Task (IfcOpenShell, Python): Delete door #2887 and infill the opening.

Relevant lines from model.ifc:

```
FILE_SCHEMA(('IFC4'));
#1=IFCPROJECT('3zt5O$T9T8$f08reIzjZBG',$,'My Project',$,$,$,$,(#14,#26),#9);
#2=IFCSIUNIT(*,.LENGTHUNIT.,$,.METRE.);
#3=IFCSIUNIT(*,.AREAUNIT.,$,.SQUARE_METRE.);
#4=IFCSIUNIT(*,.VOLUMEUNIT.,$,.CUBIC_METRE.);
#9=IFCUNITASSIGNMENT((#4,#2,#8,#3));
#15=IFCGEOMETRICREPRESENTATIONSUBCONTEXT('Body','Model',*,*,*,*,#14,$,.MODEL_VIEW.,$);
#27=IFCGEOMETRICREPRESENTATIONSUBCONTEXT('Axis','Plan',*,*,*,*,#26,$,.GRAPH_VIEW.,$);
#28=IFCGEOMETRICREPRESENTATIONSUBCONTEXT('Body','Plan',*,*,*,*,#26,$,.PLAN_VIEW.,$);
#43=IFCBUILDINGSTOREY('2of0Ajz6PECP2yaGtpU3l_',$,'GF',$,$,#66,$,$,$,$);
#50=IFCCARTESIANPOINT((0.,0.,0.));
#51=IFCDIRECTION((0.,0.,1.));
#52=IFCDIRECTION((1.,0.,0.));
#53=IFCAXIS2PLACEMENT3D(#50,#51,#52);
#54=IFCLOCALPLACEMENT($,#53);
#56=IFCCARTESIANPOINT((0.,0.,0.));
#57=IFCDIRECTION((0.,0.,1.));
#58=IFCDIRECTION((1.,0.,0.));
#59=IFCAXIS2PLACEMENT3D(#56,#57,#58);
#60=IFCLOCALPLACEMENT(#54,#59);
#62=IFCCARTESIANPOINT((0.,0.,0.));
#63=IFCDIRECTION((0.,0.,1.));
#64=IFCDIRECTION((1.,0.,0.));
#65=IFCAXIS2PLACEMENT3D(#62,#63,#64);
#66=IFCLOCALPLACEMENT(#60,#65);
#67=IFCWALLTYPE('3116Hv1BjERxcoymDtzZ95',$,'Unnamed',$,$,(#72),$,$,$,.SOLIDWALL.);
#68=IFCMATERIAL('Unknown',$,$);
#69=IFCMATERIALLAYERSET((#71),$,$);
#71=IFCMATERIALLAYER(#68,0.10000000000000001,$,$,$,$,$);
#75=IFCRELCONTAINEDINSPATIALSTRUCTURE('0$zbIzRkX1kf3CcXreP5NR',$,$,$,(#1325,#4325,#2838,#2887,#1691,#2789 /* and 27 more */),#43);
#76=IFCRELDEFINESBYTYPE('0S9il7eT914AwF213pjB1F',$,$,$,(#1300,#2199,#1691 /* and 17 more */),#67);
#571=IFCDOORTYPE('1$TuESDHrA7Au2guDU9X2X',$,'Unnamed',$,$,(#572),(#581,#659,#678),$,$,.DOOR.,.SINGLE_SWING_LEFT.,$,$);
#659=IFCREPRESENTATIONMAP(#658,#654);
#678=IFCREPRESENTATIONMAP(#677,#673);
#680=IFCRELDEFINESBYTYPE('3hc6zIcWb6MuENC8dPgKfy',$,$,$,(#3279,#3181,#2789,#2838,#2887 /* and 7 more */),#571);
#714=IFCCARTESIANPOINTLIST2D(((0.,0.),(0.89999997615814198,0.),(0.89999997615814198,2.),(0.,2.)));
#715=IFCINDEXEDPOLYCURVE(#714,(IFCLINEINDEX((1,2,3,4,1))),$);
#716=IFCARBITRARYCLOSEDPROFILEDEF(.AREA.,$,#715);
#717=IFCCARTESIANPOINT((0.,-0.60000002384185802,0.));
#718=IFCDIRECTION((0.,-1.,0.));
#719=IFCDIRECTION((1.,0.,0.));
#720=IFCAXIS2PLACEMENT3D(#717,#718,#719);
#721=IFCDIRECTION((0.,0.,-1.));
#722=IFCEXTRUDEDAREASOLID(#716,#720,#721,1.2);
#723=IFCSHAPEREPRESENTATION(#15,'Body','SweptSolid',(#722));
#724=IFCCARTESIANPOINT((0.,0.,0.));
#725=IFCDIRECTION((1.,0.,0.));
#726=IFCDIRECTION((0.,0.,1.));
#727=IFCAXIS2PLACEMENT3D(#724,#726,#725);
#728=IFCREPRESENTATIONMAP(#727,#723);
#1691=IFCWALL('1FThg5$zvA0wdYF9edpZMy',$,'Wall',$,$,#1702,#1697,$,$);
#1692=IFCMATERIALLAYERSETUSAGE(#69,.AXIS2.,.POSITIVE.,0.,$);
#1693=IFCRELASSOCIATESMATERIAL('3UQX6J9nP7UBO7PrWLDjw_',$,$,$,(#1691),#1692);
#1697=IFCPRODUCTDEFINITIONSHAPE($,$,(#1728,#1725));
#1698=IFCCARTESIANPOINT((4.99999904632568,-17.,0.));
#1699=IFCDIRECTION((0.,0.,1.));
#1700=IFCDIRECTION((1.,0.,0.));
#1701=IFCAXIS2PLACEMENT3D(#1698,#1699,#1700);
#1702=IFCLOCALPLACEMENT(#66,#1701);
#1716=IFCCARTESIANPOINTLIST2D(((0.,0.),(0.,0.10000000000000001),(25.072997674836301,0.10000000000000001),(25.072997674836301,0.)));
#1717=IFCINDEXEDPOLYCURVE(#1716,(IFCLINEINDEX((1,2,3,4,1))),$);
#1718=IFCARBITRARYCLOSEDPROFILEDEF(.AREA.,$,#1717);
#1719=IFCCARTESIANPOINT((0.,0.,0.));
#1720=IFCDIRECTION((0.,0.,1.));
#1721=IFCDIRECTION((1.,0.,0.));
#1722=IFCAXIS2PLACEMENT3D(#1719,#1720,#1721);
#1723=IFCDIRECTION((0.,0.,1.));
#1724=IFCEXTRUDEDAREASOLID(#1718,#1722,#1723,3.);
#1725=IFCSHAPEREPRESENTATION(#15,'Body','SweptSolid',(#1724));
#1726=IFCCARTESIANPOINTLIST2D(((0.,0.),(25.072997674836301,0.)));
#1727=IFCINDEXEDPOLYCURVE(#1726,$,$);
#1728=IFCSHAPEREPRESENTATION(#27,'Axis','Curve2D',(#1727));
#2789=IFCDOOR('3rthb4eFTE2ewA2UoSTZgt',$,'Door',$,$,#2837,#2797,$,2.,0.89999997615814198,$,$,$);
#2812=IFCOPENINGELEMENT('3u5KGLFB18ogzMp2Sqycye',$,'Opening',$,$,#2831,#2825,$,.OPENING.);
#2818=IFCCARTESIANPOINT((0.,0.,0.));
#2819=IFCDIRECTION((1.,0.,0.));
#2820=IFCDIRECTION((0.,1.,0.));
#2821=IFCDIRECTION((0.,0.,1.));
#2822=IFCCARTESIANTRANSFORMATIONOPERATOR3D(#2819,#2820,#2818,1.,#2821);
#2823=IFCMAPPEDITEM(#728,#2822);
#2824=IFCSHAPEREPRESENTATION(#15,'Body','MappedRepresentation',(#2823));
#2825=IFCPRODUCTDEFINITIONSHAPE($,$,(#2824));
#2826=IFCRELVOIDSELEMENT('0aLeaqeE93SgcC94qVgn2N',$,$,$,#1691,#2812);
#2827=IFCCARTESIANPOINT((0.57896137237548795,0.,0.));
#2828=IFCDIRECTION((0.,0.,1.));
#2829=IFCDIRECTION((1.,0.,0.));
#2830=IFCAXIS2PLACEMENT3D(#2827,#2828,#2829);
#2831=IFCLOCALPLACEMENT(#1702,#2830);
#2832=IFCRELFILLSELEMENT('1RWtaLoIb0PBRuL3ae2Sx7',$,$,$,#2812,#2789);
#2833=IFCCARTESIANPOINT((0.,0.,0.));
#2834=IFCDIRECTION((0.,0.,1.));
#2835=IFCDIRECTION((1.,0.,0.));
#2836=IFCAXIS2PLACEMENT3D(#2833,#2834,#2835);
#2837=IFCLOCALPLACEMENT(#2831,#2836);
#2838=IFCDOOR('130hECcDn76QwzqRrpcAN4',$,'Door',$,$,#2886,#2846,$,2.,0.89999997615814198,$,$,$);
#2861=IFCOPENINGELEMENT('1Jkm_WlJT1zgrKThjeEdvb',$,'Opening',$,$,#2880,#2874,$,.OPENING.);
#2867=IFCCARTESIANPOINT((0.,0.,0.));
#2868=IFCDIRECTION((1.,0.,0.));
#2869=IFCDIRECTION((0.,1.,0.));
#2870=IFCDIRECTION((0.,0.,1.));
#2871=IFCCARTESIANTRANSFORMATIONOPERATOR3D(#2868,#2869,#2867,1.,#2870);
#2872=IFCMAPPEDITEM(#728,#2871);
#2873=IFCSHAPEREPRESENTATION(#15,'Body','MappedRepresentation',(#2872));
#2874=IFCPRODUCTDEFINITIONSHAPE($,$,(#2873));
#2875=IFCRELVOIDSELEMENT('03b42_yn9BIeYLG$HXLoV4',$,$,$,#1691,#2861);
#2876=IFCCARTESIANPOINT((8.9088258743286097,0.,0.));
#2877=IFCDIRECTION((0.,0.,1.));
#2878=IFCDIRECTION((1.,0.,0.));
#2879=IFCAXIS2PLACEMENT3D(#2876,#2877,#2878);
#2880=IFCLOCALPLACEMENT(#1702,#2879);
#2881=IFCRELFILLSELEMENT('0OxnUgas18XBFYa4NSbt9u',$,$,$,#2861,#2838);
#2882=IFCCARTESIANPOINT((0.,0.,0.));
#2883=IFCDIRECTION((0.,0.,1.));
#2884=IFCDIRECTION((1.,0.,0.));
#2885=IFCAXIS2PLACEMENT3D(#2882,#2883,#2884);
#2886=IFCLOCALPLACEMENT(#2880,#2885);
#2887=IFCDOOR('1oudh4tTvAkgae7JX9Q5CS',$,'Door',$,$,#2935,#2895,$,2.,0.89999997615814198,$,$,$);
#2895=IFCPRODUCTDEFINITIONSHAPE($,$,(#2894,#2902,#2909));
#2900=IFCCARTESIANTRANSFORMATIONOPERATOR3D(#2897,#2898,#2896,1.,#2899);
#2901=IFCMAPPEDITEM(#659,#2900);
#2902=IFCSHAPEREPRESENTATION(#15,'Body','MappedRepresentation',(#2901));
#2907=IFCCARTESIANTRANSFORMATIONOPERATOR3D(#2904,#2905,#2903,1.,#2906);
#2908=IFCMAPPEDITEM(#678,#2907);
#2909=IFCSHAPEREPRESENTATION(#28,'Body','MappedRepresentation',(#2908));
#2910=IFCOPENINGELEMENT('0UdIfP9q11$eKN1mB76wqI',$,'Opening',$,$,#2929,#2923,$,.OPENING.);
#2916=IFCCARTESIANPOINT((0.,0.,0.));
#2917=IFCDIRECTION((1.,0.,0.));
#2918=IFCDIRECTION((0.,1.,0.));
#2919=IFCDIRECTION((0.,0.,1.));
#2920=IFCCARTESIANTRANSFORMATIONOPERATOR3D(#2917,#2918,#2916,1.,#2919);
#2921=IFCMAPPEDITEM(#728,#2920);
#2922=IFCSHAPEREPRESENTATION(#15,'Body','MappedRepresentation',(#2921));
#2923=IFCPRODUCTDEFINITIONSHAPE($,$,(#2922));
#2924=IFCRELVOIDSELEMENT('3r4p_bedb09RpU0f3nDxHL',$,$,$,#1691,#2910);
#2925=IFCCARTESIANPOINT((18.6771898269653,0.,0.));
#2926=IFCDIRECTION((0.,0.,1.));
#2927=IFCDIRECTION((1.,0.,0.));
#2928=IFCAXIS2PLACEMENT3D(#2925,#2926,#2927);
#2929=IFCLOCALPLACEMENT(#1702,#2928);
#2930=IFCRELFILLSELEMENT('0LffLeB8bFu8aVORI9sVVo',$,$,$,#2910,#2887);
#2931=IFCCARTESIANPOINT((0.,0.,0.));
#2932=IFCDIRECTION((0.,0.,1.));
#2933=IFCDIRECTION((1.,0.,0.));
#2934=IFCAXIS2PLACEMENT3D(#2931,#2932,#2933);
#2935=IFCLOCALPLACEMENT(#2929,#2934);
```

```python
import ifcopenshell
import ifcopenshell.api.feature
import ifcopenshell.api.root
import ifcopenshell.geom
import ifcopenshell.util.shape

model = ifcopenshell.open("model.ifc")
settings = ifcopenshell.geom.settings()


def volume(element):
    """Net volume in cubic metres, openings subtracted."""
    shape = ifcopenshell.geom.create_shape(settings, element)
    return ifcopenshell.util.shape.get_volume(shape.geometry)


door = model.by_guid("1oudh4tTvAkgae7JX9Q5CS")
opening = door.FillsVoids[0].RelatingOpeningElement
wall = opening.VoidsElements[0].RelatingBuildingElement
before = volume(wall)

ifcopenshell.api.root.remove_product(model, product=door)
ifcopenshell.api.feature.remove_feature(model, feature=opening)

after = volume(wall)

print(f"wall volume {before:.3f} -> {after:.3f} m3")

model.write("model_v2.ifc")
```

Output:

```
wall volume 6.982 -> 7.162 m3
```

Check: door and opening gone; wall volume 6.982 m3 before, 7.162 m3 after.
